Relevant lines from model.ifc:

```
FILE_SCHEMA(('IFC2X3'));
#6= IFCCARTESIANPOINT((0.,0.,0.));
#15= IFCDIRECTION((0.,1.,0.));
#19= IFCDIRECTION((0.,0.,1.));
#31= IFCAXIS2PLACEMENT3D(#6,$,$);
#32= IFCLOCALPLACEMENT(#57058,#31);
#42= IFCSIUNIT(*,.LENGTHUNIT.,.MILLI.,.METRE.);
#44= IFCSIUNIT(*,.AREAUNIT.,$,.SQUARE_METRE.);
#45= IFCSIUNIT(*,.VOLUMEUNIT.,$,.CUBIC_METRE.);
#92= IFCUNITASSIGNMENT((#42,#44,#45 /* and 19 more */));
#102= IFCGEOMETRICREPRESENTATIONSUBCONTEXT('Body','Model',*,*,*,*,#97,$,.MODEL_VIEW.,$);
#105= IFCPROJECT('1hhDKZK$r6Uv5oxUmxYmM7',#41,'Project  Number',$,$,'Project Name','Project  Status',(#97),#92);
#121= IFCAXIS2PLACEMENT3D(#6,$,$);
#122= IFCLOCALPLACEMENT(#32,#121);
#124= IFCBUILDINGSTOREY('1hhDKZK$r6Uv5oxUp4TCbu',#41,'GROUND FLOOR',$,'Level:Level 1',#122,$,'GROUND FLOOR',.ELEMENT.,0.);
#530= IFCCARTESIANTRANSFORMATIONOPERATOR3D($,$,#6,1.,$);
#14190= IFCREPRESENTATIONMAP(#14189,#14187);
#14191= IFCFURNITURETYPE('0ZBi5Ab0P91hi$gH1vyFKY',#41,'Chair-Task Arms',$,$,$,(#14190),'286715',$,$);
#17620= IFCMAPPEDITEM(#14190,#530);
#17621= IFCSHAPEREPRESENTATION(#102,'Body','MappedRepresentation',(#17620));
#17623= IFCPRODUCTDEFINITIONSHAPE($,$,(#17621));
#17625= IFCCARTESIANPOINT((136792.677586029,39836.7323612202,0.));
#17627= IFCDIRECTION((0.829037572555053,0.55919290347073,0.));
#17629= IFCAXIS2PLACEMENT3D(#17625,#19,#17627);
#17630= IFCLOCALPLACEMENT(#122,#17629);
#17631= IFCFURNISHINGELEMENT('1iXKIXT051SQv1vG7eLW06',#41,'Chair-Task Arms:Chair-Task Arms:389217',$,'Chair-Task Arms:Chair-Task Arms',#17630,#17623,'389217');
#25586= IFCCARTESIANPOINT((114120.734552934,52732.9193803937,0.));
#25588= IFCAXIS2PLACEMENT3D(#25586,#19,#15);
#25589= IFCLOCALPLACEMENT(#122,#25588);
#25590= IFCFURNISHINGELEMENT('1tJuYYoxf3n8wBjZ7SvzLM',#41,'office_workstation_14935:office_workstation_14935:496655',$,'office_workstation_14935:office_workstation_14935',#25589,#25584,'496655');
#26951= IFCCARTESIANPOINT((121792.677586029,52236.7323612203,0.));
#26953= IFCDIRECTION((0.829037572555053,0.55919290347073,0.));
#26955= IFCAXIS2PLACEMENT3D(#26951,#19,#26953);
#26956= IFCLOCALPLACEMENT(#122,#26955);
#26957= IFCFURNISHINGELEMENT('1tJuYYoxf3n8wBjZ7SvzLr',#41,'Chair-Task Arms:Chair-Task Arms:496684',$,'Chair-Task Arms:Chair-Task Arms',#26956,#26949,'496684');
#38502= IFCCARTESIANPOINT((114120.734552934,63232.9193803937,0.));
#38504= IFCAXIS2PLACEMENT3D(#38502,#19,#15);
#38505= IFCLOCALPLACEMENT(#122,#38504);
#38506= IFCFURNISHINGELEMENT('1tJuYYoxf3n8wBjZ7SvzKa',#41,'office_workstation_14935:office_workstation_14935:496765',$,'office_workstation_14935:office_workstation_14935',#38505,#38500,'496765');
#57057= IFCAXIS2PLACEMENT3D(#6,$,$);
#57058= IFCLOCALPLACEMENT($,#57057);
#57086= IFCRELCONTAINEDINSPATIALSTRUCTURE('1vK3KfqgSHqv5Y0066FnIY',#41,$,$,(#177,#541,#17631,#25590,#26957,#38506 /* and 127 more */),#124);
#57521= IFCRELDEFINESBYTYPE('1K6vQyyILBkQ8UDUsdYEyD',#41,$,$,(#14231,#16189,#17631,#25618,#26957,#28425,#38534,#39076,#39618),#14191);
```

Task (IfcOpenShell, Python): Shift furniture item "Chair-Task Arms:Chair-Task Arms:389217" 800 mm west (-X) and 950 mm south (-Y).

```python
import ifcopenshell
import ifcopenshell.api.geometry
import ifcopenshell.util.placement
import ifcopenshell.util.unit

model = ifcopenshell.open("model.ifc")
unit_scale = ifcopenshell.util.unit.calculate_unit_scale(model)

item = model.by_guid("1iXKIXT051SQv1vG7eLW06")
matrix = ifcopenshell.util.placement.get_local_placement(item.ObjectPlacement)
matrix[0, 3] -= 0.8 / unit_scale
matrix[1, 3] -= 0.95 / unit_scale
ifcopenshell.api.geometry.edit_object_placement(model, product=item, matrix=matrix, is_si=False)

print(ifcopenshell.util.placement.get_local_placement(item.ObjectPlacement).round(3) + 0.0)

model.write("model_v2.ifc")
```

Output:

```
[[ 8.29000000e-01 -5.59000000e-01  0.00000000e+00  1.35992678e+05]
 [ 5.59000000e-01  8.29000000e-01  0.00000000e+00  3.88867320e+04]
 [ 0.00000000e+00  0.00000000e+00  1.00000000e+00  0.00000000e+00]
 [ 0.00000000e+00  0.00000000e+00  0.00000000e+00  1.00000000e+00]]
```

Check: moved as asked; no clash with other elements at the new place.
